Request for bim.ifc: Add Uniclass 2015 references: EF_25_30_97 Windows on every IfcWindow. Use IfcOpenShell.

First a look at what the model holds.

```python
import ifcopenshell

model = ifcopenshell.open("bim.ifc")
print(model.schema)
print("classifications:", [c.Name for c in model.by_type("IfcClassification")])
for ifc_class in ("IfcDoor", "IfcRoof", "IfcStair", "IfcWall", "IfcWindow"):
    print(ifc_class, len(model.by_type(ifc_class)))
```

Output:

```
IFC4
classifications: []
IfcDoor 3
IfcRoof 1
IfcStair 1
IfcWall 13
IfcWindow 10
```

```python
import ifcopenshell
import ifcopenshell.api.classification

model = ifcopenshell.open("bim.ifc")

system = ifcopenshell.api.classification.add_classification(model, classification="Uniclass 2015")

codes = {
    "IfcWindow": ("EF_25_30_97", "Windows"),
}
for ifc_class, (code, name) in codes.items():
    products = model.by_type(ifc_class)
    ifcopenshell.api.classification.add_reference(
        model, products=products, classification=system, identification=code, name=name
    )
    print(code, len(products))

model.write("bim_v2.ifc")
```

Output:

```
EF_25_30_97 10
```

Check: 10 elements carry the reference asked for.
